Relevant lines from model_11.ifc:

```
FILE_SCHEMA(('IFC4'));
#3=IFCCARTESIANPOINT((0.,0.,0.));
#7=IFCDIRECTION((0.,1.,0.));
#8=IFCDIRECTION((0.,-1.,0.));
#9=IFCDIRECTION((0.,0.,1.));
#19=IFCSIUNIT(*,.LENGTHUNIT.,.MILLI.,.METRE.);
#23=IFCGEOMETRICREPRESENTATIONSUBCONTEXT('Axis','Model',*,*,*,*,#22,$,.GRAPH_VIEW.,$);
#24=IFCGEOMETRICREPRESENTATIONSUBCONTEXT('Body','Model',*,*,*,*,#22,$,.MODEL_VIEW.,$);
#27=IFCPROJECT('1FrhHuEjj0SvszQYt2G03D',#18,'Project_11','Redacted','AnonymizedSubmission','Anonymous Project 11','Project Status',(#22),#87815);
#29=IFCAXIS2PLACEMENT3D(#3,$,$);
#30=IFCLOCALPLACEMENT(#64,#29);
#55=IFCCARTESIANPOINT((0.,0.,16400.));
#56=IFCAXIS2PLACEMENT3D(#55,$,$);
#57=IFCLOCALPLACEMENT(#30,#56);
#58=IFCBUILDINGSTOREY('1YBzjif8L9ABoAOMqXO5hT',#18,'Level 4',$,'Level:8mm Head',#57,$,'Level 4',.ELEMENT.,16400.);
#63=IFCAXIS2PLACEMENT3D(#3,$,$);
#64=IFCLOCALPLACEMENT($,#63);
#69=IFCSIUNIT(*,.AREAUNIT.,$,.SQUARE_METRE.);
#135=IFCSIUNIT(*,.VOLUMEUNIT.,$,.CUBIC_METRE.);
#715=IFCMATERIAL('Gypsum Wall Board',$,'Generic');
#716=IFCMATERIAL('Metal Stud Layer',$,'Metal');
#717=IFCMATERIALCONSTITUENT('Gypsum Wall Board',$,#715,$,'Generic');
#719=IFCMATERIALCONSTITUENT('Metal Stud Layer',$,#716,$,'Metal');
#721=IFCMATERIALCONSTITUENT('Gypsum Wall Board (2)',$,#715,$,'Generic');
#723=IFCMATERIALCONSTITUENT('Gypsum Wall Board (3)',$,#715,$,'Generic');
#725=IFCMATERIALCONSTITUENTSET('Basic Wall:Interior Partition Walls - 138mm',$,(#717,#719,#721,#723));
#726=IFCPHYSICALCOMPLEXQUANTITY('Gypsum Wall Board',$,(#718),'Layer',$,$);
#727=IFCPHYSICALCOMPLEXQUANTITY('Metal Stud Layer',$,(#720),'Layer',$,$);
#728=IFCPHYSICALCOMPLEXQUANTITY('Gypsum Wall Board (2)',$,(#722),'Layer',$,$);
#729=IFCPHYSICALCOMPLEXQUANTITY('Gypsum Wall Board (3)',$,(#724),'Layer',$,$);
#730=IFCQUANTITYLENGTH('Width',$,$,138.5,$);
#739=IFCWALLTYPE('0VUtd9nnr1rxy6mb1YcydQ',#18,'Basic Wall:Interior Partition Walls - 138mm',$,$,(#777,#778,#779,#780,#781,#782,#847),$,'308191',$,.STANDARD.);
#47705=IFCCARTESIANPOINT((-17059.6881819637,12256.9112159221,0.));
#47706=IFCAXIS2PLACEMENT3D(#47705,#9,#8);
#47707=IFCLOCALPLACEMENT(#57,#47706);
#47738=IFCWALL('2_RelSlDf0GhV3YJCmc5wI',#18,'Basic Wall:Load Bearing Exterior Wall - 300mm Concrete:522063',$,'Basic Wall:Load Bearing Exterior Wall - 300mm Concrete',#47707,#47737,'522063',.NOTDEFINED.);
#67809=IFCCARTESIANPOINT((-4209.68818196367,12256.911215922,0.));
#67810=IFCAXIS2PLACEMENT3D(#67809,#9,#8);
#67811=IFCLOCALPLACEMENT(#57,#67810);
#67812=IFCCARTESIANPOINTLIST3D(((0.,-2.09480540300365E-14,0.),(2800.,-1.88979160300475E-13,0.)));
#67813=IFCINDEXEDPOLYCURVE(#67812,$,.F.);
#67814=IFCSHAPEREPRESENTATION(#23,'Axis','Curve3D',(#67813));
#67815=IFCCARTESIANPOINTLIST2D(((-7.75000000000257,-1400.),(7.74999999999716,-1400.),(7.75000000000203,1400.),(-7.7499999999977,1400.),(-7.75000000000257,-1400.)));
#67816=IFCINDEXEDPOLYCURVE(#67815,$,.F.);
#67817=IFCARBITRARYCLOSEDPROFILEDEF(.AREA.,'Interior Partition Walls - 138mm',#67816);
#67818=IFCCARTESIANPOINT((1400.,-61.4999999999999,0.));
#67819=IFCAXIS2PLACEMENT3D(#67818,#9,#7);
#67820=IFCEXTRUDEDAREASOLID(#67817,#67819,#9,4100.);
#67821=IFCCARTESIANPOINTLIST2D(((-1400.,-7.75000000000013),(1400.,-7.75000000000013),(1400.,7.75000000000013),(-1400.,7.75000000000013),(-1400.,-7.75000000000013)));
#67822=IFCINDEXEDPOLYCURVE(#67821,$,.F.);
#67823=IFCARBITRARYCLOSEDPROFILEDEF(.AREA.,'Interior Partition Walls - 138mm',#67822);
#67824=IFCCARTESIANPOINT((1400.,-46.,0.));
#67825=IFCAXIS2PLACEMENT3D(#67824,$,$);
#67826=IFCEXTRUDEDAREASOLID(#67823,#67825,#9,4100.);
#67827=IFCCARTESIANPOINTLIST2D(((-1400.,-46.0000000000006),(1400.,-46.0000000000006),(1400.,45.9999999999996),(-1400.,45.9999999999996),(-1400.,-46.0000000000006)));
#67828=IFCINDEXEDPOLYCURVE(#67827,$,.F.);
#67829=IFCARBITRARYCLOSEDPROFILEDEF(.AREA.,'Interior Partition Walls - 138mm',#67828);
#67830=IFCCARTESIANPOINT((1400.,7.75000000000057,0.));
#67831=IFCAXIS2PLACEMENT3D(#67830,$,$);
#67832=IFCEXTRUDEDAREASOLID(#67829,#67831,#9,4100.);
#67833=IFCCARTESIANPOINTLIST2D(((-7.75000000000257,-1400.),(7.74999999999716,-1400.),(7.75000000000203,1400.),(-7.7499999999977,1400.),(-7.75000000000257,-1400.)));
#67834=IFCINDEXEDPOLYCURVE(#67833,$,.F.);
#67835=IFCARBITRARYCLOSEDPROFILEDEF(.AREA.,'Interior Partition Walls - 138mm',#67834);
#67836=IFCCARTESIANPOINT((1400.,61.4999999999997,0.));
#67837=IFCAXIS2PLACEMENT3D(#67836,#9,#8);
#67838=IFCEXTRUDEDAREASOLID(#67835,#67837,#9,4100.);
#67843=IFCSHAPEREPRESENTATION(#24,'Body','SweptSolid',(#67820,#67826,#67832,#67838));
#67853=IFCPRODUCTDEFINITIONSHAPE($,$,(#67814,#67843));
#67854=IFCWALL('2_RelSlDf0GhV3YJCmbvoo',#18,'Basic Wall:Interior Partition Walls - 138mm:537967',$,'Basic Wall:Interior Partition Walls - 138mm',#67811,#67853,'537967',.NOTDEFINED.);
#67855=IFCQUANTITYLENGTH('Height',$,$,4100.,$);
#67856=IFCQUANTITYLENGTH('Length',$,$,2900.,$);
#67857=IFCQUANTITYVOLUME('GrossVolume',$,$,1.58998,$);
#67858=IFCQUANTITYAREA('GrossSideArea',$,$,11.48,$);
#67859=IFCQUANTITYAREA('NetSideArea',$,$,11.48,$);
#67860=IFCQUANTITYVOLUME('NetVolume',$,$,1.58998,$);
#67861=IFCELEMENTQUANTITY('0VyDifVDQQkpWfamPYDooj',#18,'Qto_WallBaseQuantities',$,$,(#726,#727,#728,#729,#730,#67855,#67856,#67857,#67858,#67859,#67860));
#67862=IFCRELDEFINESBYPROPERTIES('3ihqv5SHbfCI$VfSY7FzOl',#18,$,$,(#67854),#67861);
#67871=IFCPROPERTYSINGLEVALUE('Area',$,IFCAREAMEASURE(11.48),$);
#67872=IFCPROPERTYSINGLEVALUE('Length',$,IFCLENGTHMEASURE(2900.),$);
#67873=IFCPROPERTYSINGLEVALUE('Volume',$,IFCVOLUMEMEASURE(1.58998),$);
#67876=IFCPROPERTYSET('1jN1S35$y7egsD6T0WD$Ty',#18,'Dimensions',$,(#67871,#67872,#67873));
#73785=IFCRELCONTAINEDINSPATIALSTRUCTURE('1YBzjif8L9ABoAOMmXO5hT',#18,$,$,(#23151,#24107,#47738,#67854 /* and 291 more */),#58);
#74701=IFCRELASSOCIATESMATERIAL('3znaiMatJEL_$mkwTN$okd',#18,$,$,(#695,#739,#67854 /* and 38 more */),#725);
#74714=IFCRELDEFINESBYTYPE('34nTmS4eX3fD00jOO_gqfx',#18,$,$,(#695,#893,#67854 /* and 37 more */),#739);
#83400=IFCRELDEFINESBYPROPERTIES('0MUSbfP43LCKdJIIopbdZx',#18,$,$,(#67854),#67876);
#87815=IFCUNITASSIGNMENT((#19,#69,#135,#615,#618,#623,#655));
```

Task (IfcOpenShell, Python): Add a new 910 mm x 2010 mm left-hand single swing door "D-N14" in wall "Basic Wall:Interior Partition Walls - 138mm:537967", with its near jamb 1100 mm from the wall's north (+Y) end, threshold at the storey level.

```python
import numpy as np
import ifcopenshell
import ifcopenshell.api.feature
import ifcopenshell.api.geometry
import ifcopenshell.api.pset
import ifcopenshell.api.root
import ifcopenshell.api.spatial
import ifcopenshell.geom
import ifcopenshell.util.element
import ifcopenshell.util.placement
import ifcopenshell.util.representation
import ifcopenshell.util.shape
import ifcopenshell.util.unit

model = ifcopenshell.open("model_11.ifc")
unit_scale = ifcopenshell.util.unit.calculate_unit_scale(model)
area_scale = ifcopenshell.util.unit.calculate_unit_scale(model, "AREAUNIT")
volume_scale = ifcopenshell.util.unit.calculate_unit_scale(model, "VOLUMEUNIT")
settings = ifcopenshell.geom.settings()


def volume(element):
    """Net volume in cubic metres, openings subtracted."""
    shape = ifcopenshell.geom.create_shape(settings, element)
    return ifcopenshell.util.shape.get_volume(shape.geometry)


wall = model.by_id(67854)
storey = ifcopenshell.util.element.get_container(wall, ifc_class="IfcBuildingStorey")
context = ifcopenshell.util.representation.get_context(model, "Model", "Body", "MODEL_VIEW")
before = volume(wall)

width, height, from_end, sill = 0.91, 2.01, 1.1, 0.0  # metres

# The wall runs along its own X axis, and the end named is its -X end.
wall_shape = ifcopenshell.geom.create_shape(settings, wall)
x, y, z = ifcopenshell.util.shape.get_vertices(wall_shape.geometry).T
start = x.min() + from_end
face, thickness = float(y.min()), float(y.max() - y.min())
wall_matrix = ifcopenshell.util.placement.get_local_placement(wall.ObjectPlacement)
level = ifcopenshell.util.placement.get_local_placement(storey.ObjectPlacement)[2, 3]


def in_wall(x, y):
    """Placement at x, y metres in the wall's axes, at sill height."""
    matrix = wall_matrix.copy()
    matrix[:, 3] = wall_matrix @ np.array([x / unit_scale, y / unit_scale, 0.0, 1.0])
    matrix[2, 3] = level + sill / unit_scale
    return matrix


# Opening: a box that overshoots both wall faces by 50 mm.
opening = ifcopenshell.api.root.create_entity(model, ifc_class="IfcOpeningElement", predefined_type="OPENING")
box = ifcopenshell.api.geometry.add_wall_representation(
    model, context=context, length=width, height=height, thickness=thickness + 0.1
)
ifcopenshell.api.geometry.assign_representation(model, product=opening, representation=box)
ifcopenshell.api.geometry.edit_object_placement(model, product=opening, matrix=in_wall(start, face - 0.05), is_si=False)
ifcopenshell.api.feature.add_feature(model, feature=opening, element=wall)

door = ifcopenshell.api.root.create_entity(model, ifc_class="IfcDoor", name="D-N14", predefined_type="DOOR")
door.OverallWidth, door.OverallHeight = width / unit_scale, height / unit_scale
door.OperationType = "SINGLE_SWING_LEFT"
body = ifcopenshell.api.geometry.add_door_representation(
    model,
    context=context,
    overall_width=door.OverallWidth,
    overall_height=door.OverallHeight,
    operation_type="SINGLE_SWING_LEFT",
    lining_properties={"LiningDepth": thickness / unit_scale, "ThresholdDepth": thickness / unit_scale},
)
ifcopenshell.api.geometry.assign_representation(model, product=door, representation=body)
ifcopenshell.api.spatial.assign_container(model, products=[door], relating_structure=storey)
ifcopenshell.api.feature.add_filling(model, opening=opening, element=door)

# The lining spans the wall, so the door starts at the wall face.
ifcopenshell.api.geometry.edit_object_placement(model, product=door, matrix=in_wall(start, face), is_si=False)

after = volume(wall)

# Update the wall's stored quantities.
qto = model.by_id(ifcopenshell.util.element.get_pset(wall, "Qto_WallBaseQuantities", should_inherit=False)["id"])
ifcopenshell.api.pset.edit_qto(model, qto=qto, properties={
    "NetSideArea": after / thickness / area_scale,
    "NetVolume": after / volume_scale,
})
pset = model.by_id(ifcopenshell.util.element.get_pset(wall, "Dimensions", should_inherit=False)["id"])
ifcopenshell.api.pset.edit_pset(model, pset=pset, properties={
    "Area": model.create_entity("IfcAreaMeasure", after / thickness / area_scale),
    "Volume": model.create_entity("IfcVolumeMeasure", after / volume_scale),
})

print(f"wall volume {before:.3f} -> {after:.3f} m3")

model.write("model_11-out.ifc")
```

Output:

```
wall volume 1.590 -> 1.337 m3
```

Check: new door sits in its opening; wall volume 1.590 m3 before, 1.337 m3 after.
